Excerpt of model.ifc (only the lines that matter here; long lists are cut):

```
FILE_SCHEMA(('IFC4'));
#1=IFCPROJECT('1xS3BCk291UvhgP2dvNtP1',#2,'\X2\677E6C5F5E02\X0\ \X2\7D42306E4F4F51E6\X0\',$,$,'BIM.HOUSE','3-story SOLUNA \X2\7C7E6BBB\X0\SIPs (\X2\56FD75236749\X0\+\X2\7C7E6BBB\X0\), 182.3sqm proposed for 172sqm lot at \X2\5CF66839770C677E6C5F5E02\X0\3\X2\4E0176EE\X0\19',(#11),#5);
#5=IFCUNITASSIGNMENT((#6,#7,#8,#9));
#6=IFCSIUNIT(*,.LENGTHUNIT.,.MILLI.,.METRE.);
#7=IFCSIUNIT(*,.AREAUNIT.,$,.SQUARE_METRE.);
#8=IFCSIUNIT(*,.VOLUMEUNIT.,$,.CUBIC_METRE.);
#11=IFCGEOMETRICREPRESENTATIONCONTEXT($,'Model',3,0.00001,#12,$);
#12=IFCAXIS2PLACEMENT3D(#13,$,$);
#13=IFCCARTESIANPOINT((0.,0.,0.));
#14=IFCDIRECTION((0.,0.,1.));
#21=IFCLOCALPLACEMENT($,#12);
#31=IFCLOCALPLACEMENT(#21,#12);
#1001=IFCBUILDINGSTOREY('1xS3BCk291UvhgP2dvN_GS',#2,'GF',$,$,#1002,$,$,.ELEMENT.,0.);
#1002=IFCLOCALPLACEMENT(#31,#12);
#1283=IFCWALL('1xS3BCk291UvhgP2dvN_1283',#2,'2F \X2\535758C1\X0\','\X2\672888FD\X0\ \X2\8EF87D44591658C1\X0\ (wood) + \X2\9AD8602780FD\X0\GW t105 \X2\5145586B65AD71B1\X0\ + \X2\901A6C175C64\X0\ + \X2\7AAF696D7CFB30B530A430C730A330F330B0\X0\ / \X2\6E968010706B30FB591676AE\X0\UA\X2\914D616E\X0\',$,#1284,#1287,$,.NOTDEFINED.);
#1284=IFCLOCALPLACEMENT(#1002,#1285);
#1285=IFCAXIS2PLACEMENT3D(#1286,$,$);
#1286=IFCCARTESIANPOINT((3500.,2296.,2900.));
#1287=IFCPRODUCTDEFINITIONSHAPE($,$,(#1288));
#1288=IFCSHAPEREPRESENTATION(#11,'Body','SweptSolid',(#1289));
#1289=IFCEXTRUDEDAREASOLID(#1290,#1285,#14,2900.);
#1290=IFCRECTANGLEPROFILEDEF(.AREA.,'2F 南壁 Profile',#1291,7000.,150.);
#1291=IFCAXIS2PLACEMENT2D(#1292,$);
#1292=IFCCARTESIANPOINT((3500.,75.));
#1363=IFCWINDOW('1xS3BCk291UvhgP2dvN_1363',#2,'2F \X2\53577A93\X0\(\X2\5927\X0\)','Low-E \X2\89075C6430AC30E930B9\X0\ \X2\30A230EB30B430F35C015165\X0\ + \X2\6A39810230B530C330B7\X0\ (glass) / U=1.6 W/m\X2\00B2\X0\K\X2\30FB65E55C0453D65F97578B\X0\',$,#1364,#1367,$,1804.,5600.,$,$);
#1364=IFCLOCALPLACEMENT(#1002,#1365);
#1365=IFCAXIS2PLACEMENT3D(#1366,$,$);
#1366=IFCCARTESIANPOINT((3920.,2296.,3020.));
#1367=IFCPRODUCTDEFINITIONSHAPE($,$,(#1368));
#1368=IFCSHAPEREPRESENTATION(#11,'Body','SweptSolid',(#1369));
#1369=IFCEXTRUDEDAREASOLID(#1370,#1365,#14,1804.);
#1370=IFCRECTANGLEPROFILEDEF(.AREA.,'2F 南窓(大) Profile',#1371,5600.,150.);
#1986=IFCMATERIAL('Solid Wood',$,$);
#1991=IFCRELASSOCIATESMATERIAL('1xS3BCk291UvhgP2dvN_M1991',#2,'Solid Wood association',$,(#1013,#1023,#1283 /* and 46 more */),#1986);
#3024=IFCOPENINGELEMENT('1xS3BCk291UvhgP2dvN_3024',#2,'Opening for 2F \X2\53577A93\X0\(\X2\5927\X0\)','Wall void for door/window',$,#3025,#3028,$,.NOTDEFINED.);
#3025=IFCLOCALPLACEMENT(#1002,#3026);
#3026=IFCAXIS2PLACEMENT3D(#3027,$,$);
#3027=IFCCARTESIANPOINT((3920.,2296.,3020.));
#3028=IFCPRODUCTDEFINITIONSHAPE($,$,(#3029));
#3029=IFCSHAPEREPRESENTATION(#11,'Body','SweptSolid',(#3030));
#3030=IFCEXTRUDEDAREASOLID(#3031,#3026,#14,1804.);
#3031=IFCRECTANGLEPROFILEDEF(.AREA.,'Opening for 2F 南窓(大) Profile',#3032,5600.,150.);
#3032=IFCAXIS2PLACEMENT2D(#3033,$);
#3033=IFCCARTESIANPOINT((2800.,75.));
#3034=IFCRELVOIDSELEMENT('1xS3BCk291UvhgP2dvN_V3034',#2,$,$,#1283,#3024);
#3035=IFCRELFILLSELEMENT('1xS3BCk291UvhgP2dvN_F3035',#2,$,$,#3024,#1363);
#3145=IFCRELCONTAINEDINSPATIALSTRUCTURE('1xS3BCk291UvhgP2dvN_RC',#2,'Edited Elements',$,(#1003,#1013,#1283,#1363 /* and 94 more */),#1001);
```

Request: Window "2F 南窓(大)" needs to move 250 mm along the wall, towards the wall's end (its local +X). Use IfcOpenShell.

```python
import ifcopenshell
import ifcopenshell.api.geometry
import ifcopenshell.util.placement

model = ifcopenshell.open("model.ifc")

window = model.by_guid("1xS3BCk291UvhgP2dvN_1363")
opening = window.FillsVoids[0].RelatingOpeningElement
wall = opening.VoidsElements[0].RelatingBuildingElement

wall_matrix = ifcopenshell.util.placement.get_local_placement(wall.ObjectPlacement)
shift = wall_matrix[:3, 0] * 250.0
before = ifcopenshell.util.placement.get_local_placement(window.ObjectPlacement)[:3, 3].copy()

# The window is not placed relative to its opening, so move both.
for product in (opening, window):
    matrix = ifcopenshell.util.placement.get_local_placement(product.ObjectPlacement)
    matrix[:3, 3] += shift
    ifcopenshell.api.geometry.edit_object_placement(model, product=product, matrix=matrix, is_si=False)

after = ifcopenshell.util.placement.get_local_placement(window.ObjectPlacement)[:3, 3]
print("window moved by", (after - before).round(3) + 0.0)

model.write("model_rev.ifc")
```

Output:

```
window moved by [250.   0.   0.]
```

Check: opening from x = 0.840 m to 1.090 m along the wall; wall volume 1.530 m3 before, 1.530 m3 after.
